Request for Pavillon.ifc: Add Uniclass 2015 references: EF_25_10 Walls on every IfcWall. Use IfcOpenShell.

First a look at what the model holds.

```python
import ifcopenshell

model = ifcopenshell.open("Pavillon.ifc")
print(model.schema)
print("classifications:", [c.Name for c in model.by_type("IfcClassification")])
for ifc_class in ("IfcDoor", "IfcRoof", "IfcStair", "IfcWall", "IfcWindow"):
    print(ifc_class, len(model.by_type(ifc_class)))
```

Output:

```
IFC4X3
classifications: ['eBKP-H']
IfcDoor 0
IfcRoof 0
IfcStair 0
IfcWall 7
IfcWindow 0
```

```python
import ifcopenshell
import ifcopenshell.api.classification

model = ifcopenshell.open("Pavillon.ifc")

system = ifcopenshell.api.classification.add_classification(model, classification="Uniclass 2015")

codes = {
    "IfcWall": ("EF_25_10", "Walls"),
}
for ifc_class, (code, name) in codes.items():
    products = model.by_type(ifc_class)
    ifcopenshell.api.classification.add_reference(
        model, products=products, classification=system, identification=code, name=name
    )
    print(code, len(products))

model.write("Pavillon-out.ifc")
```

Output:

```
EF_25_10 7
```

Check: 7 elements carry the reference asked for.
